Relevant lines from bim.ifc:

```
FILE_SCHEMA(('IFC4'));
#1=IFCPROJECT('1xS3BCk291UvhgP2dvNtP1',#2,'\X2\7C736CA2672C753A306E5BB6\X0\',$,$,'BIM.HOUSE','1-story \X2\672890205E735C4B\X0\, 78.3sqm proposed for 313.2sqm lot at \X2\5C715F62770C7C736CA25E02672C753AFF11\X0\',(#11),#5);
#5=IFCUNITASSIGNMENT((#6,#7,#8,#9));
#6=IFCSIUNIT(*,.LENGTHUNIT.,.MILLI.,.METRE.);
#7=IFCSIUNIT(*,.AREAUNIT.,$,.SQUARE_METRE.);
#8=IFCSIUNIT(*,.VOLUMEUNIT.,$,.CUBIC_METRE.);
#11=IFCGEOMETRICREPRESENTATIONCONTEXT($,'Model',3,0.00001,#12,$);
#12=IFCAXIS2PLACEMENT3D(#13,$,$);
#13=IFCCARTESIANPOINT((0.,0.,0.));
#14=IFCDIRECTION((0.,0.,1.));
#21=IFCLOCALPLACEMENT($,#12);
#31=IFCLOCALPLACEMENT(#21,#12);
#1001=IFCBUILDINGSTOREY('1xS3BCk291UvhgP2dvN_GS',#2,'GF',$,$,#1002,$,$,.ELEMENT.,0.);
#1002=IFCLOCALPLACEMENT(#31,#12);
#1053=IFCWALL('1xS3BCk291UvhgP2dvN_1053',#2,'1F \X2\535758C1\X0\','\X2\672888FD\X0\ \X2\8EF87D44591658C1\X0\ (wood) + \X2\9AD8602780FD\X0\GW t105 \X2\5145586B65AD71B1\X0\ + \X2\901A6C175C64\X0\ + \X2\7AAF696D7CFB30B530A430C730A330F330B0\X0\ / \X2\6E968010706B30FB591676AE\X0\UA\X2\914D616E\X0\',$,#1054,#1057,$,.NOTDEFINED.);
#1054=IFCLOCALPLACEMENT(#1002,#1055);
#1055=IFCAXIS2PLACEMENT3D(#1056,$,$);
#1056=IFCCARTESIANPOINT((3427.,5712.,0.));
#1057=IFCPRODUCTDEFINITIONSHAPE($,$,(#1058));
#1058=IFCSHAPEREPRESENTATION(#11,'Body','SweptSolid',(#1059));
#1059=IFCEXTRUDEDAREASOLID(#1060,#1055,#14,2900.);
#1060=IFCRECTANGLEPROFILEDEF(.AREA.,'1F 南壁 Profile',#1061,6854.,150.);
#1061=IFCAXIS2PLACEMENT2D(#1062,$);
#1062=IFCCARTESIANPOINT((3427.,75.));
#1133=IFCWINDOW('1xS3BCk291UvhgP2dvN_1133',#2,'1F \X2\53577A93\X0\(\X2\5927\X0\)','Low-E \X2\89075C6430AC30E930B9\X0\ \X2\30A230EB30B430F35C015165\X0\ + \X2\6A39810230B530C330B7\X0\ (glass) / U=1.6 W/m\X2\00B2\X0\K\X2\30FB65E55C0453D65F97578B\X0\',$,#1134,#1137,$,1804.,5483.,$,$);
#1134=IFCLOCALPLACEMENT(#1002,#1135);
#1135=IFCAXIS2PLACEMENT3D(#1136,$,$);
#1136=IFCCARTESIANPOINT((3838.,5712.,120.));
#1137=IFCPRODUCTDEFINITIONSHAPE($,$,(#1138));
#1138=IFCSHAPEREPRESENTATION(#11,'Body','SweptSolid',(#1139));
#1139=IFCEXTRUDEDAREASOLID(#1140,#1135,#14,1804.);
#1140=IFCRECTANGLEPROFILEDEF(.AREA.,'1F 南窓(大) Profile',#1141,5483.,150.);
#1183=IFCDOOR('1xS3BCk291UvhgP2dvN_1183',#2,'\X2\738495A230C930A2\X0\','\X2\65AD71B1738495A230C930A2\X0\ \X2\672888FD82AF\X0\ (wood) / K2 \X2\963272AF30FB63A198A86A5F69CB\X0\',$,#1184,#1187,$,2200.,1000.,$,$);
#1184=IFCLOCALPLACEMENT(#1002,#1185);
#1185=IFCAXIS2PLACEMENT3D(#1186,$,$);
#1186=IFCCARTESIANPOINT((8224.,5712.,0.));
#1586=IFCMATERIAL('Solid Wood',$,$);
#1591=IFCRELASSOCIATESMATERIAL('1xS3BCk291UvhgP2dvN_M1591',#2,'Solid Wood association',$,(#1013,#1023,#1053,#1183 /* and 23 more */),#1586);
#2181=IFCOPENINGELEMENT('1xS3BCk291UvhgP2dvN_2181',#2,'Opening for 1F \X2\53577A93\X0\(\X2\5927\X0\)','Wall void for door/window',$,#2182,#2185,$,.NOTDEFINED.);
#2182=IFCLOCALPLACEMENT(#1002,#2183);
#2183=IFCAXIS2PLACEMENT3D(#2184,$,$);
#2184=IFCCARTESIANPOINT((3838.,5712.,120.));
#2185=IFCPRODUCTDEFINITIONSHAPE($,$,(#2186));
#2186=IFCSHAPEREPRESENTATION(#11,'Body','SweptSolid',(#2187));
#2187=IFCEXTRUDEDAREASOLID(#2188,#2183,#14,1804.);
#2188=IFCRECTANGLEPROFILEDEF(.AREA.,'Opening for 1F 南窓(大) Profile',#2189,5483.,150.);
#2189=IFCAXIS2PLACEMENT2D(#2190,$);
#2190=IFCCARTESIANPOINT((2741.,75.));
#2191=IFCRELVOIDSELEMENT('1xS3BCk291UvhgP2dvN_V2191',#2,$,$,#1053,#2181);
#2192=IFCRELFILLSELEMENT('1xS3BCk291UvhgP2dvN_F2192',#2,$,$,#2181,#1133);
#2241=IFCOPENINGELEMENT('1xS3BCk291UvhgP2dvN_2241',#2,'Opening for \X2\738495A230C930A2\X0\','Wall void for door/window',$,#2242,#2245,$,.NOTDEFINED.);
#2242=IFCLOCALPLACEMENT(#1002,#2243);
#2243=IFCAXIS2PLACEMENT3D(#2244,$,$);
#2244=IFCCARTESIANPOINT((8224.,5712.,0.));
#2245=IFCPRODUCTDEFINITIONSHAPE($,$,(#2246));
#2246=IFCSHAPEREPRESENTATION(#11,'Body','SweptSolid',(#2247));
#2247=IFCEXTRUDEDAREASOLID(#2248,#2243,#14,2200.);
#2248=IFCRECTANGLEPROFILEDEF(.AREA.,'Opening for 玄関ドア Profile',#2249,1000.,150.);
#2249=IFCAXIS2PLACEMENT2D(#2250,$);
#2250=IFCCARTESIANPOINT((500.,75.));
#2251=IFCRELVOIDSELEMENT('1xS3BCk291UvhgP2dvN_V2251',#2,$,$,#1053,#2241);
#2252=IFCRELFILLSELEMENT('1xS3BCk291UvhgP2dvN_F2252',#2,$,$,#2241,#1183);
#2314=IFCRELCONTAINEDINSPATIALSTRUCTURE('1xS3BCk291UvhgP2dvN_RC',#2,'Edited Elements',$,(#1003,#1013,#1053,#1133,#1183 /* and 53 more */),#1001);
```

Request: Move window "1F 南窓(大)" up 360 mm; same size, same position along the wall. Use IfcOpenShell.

```python
import numpy as np
import ifcopenshell
import ifcopenshell.api.geometry
import ifcopenshell.util.placement
import ifcopenshell.util.unit

model = ifcopenshell.open("bim.ifc")
unit_scale = ifcopenshell.util.unit.calculate_unit_scale(model)

window = model.by_guid("1xS3BCk291UvhgP2dvN_1133")
opening = window.FillsVoids[0].RelatingOpeningElement
dz = 360.0

shift = np.array([0.0, 0.0, dz])
# The window is not placed relative to its opening, so move both.
for product in (opening, window):
    matrix = ifcopenshell.util.placement.get_local_placement(product.ObjectPlacement)
    matrix[:3, 3] += shift
    ifcopenshell.api.geometry.edit_object_placement(model, product=product, matrix=matrix, is_si=False)

print(f"moved by {dz * unit_scale:+.3f} m")

model.write("bim_edited.ifc")
```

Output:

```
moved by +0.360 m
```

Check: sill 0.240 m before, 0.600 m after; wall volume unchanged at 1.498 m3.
